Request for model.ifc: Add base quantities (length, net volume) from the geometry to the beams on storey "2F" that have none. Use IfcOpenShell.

First a look at what the model holds.

```python
import ifcopenshell
import ifcopenshell.util.element
import ifcopenshell.util.unit

model = ifcopenshell.open("model.ifc")
print(model.schema)
for unit_type in ("LENGTHUNIT", "AREAUNIT", "VOLUMEUNIT"):
    print(unit_type, ifcopenshell.util.unit.calculate_unit_scale(model, unit_type))
storey = next(s for s in model.by_type("IfcBuildingStorey") if s.Name == "2F")
beams = [e for e in ifcopenshell.util.element.get_decomposition(storey) if e.is_a("IfcBeam")]
for e in sorted(beams, key=lambda e: e.id()):
    print(e.id(), e.is_a(), e.Name, list(ifcopenshell.util.element.get_psets(e, qtos_only=True)), sep=" | ")
```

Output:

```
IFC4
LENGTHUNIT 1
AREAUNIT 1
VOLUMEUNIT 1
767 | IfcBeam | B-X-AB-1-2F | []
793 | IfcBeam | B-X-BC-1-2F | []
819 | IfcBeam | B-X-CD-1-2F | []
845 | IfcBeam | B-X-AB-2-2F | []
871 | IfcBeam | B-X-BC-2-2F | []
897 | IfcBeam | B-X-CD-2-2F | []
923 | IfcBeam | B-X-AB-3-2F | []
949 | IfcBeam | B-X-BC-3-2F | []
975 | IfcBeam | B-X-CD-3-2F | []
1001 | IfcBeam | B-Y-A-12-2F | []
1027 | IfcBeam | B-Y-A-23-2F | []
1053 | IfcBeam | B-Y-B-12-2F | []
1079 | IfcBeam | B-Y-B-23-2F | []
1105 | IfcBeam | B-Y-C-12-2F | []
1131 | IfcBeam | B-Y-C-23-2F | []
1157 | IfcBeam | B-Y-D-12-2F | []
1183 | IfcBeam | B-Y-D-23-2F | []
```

```python
import ifcopenshell
import ifcopenshell.api.pset
import ifcopenshell.geom
import ifcopenshell.util.element
import ifcopenshell.util.shape
import ifcopenshell.util.unit

model = ifcopenshell.open("model.ifc")
unit_scale = ifcopenshell.util.unit.calculate_unit_scale(model)
volume_scale = ifcopenshell.util.unit.calculate_unit_scale(model, "VOLUMEUNIT")
settings = ifcopenshell.geom.settings()

storey = next(s for s in model.by_type("IfcBuildingStorey") if s.Name == "2F")
beams = [e for e in ifcopenshell.util.element.get_decomposition(storey) if e.is_a("IfcBeam")]

for e in sorted(beams, key=lambda e: e.id()):
    if ifcopenshell.util.element.get_psets(e, qtos_only=True, should_inherit=False):
        continue
    # Geometry comes back in metres, in the element's own axes.
    shape = ifcopenshell.geom.create_shape(settings, e)
    values = {
        "Length": ifcopenshell.util.shape.get_max_xyz(shape.geometry) / unit_scale,
        "NetVolume": ifcopenshell.util.shape.get_volume(shape.geometry) / volume_scale,
    }
    qto = ifcopenshell.api.pset.add_qto(model, product=e, name="Qto_BeamBaseQuantities")
    ifcopenshell.api.pset.edit_qto(model, qto=qto, properties=values)
    print(e.id(), {k: round(v, 3) for k, v in values.items()})

model.write("model_v2.ifc")
```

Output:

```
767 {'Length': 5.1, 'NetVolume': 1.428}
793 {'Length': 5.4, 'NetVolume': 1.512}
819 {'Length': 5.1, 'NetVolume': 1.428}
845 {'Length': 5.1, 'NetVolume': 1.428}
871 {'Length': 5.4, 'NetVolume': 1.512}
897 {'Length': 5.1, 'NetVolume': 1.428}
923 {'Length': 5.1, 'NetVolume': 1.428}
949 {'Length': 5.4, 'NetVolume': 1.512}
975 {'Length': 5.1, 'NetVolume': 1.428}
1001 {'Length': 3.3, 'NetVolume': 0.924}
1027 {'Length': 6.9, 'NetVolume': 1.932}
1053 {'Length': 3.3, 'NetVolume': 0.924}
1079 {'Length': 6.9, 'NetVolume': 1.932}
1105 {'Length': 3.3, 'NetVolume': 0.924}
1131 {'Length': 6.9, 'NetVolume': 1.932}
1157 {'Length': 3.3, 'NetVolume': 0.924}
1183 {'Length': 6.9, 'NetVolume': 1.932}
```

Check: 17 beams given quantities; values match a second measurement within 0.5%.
